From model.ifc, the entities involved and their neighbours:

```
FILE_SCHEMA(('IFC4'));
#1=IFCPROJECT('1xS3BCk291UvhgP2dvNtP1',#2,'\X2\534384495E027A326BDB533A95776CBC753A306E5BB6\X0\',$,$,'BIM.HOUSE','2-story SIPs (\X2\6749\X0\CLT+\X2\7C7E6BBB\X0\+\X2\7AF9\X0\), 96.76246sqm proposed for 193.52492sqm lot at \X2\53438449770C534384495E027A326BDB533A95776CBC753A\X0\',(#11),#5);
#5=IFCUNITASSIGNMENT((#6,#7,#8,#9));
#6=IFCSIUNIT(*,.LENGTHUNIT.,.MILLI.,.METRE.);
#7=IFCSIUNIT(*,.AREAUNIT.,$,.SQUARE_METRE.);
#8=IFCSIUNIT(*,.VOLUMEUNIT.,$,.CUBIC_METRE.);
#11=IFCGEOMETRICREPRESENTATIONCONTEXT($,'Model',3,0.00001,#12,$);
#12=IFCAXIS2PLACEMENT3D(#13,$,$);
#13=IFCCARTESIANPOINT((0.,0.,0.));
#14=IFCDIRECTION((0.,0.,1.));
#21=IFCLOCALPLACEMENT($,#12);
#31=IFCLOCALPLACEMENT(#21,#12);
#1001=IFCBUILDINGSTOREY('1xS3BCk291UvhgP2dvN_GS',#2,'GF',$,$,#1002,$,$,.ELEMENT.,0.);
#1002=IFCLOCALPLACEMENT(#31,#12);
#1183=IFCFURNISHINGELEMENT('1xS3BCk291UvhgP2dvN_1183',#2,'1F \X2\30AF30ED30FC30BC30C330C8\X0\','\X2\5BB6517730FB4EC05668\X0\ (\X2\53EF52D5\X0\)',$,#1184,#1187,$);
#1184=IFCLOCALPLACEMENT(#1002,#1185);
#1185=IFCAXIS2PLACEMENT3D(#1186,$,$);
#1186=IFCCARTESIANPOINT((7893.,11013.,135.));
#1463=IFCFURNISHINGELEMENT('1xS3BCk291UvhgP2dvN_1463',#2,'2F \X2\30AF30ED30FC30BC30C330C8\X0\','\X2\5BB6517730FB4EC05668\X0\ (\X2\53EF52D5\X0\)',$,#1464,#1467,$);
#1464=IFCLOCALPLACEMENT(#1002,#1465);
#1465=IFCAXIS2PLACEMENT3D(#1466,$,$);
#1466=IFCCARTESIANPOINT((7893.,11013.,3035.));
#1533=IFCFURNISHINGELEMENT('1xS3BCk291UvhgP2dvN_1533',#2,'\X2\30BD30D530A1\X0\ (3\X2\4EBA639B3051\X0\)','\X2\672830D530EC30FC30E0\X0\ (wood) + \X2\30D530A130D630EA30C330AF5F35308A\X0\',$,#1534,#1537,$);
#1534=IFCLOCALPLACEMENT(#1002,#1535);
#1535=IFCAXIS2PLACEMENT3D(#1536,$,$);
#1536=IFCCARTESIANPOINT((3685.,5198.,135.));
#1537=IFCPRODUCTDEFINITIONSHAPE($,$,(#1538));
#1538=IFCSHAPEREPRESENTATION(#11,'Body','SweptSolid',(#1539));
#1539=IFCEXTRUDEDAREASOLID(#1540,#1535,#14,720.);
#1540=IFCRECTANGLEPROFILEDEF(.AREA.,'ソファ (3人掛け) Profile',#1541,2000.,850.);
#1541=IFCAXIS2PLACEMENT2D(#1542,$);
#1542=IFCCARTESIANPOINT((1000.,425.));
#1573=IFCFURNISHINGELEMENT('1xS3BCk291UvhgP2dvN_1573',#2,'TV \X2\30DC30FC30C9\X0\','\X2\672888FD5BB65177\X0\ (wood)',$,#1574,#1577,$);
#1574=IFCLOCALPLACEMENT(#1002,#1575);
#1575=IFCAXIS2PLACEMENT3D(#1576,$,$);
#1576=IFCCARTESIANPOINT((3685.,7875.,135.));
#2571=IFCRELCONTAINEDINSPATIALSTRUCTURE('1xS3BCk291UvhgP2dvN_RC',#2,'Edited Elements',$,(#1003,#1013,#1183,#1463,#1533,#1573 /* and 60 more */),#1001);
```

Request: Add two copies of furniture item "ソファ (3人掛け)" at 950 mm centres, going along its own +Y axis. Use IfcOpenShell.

```python
import ifcopenshell
import ifcopenshell.api.geometry
import ifcopenshell.api.root
import ifcopenshell.util.element
import ifcopenshell.util.placement
import ifcopenshell.util.unit

model = ifcopenshell.open("model.ifc")
unit_scale = ifcopenshell.util.unit.calculate_unit_scale(model)


def reuse_history(source, copy):
    """copy_class also copies each property set's owner history, people and application; keep the originals."""
    for rel in copy.IsDefinedBy:
        if rel.is_a("IfcRelDefinesByProperties") and (history := rel.RelatingPropertyDefinition.OwnerHistory):
            rel.RelatingPropertyDefinition.OwnerHistory = source.OwnerHistory
            ifcopenshell.util.element.remove_deep2(model, history)


source = model.by_guid("1xS3BCk291UvhgP2dvN_1533")
base = ifcopenshell.util.placement.get_local_placement(source.ObjectPlacement)
step = base[:3, 1] * 0.95 / unit_scale

for i in range(1, 3):
    copy = ifcopenshell.api.root.copy_class(model, product=source)
    copy.Representation = ifcopenshell.util.element.copy_deep(
        model, source.Representation, exclude=["IfcGeometricRepresentationContext", "IfcRepresentationMap"]
    )
    reuse_history(source, copy)
    matrix = base.copy()
    matrix[:3, 3] += i * step
    print("added at", matrix[:3, 3].round(3) + 0.0)
    ifcopenshell.api.geometry.edit_object_placement(model, product=copy, matrix=matrix, is_si=False)

model.write("model_updated.ifc")
```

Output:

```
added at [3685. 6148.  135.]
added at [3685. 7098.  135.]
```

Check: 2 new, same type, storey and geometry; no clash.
